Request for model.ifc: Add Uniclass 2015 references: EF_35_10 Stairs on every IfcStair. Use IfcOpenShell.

First a look at what the model holds.

```python
import ifcopenshell

model = ifcopenshell.open("model.ifc")
print(model.schema)
print("classifications:", [c.Name for c in model.by_type("IfcClassification")])
for ifc_class in ("IfcDoor", "IfcRoof", "IfcStair", "IfcWall", "IfcWindow"):
    print(ifc_class, len(model.by_type(ifc_class)))
```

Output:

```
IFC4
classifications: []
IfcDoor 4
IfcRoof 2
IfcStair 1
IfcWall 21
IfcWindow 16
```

```python
import ifcopenshell
import ifcopenshell.api.classification

model = ifcopenshell.open("model.ifc")

system = ifcopenshell.api.classification.add_classification(model, classification="Uniclass 2015")

codes = {
    "IfcStair": ("EF_35_10", "Stairs"),
}
for ifc_class, (code, name) in codes.items():
    products = model.by_type(ifc_class)
    ifcopenshell.api.classification.add_reference(
        model, products=products, classification=system, identification=code, name=name
    )
    print(code, len(products))

model.write("model_v2.ifc")
```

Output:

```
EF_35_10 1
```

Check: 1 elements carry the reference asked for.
